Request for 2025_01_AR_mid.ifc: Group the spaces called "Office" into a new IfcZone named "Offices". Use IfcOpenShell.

First a look at what the model holds.

```python
import ifcopenshell

model = ifcopenshell.open("2025_01_AR_mid.ifc")
print(model.schema)
seen = {}
for space in model.by_type("IfcSpace"):
    seen[space.LongName] = seen.get(space.LongName, 0) + 1
for name, count in sorted(seen.items(), key=str):
    print(count, "x", name)
print("zones:", [z.Name for z in model.by_type("IfcZone")][:20])
```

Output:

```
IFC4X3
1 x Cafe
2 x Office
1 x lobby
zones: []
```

```python
import ifcopenshell
import ifcopenshell.api.group
import ifcopenshell.api.root

model = ifcopenshell.open("2025_01_AR_mid.ifc")

names = {"Office"}
spaces = [s for s in model.by_type("IfcSpace") if s.LongName in names]

zone = ifcopenshell.api.root.create_entity(model, ifc_class="IfcZone", name="Offices")
ifcopenshell.api.group.assign_group(model, products=spaces, group=zone)
print(len(spaces), "spaces in", zone.Name)

model.write("2025_01_AR_mid_updated.ifc")
```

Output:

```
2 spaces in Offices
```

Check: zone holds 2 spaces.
